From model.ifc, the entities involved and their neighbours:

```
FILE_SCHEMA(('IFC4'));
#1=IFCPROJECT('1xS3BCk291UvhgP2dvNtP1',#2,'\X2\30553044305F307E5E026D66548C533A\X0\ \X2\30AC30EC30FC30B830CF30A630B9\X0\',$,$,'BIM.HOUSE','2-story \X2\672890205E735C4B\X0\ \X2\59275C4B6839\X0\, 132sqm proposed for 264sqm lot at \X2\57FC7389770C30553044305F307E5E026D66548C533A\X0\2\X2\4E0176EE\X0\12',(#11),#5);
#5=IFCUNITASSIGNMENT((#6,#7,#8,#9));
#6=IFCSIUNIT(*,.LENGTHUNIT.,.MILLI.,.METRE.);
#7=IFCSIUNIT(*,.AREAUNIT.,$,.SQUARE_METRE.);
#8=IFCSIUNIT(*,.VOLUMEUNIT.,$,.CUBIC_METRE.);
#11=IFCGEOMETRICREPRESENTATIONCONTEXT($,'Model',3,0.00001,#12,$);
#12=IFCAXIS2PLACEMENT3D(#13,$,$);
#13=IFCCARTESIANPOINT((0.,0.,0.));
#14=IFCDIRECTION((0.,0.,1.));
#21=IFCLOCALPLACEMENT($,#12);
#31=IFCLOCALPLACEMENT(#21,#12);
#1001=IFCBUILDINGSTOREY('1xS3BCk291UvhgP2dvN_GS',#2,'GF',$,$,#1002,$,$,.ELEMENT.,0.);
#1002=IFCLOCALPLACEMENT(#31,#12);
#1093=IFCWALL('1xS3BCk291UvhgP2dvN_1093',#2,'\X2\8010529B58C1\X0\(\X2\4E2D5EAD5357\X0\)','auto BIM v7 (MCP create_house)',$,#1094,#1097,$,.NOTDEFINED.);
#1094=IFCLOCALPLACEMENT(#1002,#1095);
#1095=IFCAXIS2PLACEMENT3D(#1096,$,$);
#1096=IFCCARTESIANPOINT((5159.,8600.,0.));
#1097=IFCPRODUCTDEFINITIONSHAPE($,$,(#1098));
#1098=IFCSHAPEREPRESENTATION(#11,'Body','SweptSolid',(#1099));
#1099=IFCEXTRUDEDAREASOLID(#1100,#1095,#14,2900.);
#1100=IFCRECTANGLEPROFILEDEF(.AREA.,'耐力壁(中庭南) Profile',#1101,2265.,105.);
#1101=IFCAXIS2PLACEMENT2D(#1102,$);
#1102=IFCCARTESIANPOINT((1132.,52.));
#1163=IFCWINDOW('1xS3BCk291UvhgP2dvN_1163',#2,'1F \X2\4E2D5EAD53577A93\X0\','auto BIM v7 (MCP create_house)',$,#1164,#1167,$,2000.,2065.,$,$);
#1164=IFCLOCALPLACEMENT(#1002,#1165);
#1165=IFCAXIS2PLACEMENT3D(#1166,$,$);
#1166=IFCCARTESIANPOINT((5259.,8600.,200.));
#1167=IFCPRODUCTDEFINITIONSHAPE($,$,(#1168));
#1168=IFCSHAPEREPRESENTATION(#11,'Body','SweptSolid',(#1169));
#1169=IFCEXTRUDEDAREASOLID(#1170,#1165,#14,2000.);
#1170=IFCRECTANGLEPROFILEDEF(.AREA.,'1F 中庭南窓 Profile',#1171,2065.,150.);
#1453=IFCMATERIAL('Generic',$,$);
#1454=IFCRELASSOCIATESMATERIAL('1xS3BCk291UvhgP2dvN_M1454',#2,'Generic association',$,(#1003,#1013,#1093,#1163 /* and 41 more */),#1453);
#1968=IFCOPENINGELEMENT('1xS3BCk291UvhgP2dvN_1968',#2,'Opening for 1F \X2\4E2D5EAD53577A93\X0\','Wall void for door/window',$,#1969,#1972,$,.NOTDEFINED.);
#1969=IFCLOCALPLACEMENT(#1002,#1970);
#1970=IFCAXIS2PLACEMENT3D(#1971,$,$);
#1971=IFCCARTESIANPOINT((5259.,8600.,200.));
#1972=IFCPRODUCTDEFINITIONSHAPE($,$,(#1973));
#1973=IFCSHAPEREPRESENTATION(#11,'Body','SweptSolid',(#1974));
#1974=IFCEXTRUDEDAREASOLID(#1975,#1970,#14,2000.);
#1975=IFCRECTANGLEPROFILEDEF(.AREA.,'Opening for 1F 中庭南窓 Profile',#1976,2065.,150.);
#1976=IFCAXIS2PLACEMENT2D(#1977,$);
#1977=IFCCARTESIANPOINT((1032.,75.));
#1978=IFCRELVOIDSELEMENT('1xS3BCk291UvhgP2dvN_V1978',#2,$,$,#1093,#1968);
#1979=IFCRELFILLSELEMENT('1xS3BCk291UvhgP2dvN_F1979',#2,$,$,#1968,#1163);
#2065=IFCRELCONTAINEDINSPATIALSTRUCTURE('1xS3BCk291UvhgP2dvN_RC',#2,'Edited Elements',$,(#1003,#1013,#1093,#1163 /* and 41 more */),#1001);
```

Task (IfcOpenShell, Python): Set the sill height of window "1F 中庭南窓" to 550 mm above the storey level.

```python
import numpy as np
import ifcopenshell
import ifcopenshell.api.geometry
import ifcopenshell.geom
import ifcopenshell.util.element
import ifcopenshell.util.placement
import ifcopenshell.util.shape
import ifcopenshell.util.unit

model = ifcopenshell.open("model.ifc")
unit_scale = ifcopenshell.util.unit.calculate_unit_scale(model)

window = model.by_guid("1xS3BCk291UvhgP2dvN_1163")
opening = window.FillsVoids[0].RelatingOpeningElement
storey = ifcopenshell.util.element.get_container(window, ifc_class="IfcBuildingStorey")
level = ifcopenshell.util.placement.get_local_placement(storey.ObjectPlacement)[2, 3]

# The opening's origin need not be at the sill, so measure its lowest point.
shape = ifcopenshell.geom.create_shape(ifcopenshell.geom.settings(), opening)
bottom = ifcopenshell.util.shape.get_shape_bottom_elevation(shape, shape.geometry) / unit_scale
dz = level + 550.0 - bottom

shift = np.array([0.0, 0.0, dz])
# The window is not placed relative to its opening, so move both.
for product in (opening, window):
    matrix = ifcopenshell.util.placement.get_local_placement(product.ObjectPlacement)
    matrix[:3, 3] += shift
    ifcopenshell.api.geometry.edit_object_placement(model, product=product, matrix=matrix, is_si=False)

print(f"moved by {dz * unit_scale:+.3f} m")

model.write("model_rev.ifc")
```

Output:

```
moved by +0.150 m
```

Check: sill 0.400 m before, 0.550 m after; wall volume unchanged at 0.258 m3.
